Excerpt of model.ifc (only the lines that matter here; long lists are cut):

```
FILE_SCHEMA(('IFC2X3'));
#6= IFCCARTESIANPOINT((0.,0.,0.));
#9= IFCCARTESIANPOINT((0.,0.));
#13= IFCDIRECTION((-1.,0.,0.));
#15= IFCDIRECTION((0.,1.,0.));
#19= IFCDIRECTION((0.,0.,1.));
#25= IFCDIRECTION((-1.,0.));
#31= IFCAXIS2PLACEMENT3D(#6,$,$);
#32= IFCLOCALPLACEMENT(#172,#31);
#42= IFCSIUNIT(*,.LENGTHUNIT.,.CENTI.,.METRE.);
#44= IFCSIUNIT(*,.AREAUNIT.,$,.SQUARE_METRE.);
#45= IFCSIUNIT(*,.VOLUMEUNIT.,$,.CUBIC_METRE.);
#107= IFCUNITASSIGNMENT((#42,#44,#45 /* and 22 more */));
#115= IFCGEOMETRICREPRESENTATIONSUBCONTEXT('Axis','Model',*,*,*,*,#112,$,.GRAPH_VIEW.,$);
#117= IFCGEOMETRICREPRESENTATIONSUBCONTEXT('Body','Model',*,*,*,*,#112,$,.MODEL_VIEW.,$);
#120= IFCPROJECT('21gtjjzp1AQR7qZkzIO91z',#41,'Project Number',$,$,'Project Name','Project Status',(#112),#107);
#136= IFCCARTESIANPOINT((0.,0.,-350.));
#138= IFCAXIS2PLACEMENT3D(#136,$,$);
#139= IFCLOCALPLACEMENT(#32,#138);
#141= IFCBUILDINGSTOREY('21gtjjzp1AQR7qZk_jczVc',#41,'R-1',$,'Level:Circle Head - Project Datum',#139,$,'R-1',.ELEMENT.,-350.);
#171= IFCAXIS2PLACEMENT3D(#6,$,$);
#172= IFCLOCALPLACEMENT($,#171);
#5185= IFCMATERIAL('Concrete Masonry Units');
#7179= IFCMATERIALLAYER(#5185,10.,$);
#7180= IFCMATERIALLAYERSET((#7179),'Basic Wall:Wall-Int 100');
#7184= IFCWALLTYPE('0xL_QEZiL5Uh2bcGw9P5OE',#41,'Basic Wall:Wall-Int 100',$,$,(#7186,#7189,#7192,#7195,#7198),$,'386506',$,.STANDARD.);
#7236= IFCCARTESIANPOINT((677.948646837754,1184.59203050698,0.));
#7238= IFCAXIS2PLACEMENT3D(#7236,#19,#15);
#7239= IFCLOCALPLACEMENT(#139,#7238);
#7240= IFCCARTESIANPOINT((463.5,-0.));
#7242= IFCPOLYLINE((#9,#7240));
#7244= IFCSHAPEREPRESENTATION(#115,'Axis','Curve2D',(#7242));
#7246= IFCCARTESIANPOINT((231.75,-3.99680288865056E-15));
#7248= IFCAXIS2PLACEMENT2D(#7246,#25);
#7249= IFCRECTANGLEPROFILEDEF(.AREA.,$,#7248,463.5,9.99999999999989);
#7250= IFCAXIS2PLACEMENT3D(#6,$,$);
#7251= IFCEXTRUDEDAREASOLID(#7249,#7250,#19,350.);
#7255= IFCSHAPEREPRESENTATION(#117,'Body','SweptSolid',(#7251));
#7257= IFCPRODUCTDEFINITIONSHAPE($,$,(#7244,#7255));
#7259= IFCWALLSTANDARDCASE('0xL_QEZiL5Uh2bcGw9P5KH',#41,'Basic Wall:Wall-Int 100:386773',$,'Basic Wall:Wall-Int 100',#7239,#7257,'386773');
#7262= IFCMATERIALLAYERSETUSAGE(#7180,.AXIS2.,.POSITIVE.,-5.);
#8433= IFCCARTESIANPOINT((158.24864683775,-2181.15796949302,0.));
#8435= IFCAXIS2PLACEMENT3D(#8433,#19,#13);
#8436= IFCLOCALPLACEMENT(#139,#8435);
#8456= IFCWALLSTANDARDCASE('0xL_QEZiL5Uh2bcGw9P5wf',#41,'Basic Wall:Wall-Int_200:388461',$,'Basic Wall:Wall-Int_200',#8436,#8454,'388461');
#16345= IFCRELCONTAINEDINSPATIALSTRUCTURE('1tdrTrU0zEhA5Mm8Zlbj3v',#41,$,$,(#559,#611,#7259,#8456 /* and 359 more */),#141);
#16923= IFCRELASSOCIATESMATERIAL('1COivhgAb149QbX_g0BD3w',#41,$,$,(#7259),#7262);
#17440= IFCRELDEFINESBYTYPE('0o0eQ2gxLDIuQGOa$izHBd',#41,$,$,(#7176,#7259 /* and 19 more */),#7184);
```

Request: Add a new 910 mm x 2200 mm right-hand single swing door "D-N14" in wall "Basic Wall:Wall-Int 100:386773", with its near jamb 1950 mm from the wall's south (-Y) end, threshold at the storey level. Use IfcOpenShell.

```python
import numpy as np
import ifcopenshell
import ifcopenshell.api.feature
import ifcopenshell.api.geometry
import ifcopenshell.api.root
import ifcopenshell.api.spatial
import ifcopenshell.api.type
import ifcopenshell.geom
import ifcopenshell.util.element
import ifcopenshell.util.placement
import ifcopenshell.util.representation
import ifcopenshell.util.shape
import ifcopenshell.util.unit

model = ifcopenshell.open("model.ifc")
unit_scale = ifcopenshell.util.unit.calculate_unit_scale(model)
settings = ifcopenshell.geom.settings()


def volume(element):
    """Net volume in cubic metres, openings subtracted."""
    shape = ifcopenshell.geom.create_shape(settings, element)
    return ifcopenshell.util.shape.get_volume(shape.geometry)


wall = model.by_id(7259)
storey = ifcopenshell.util.element.get_container(wall, ifc_class="IfcBuildingStorey")
context = ifcopenshell.util.representation.get_context(model, "Model", "Body", "MODEL_VIEW")
before = volume(wall)

width, height, from_end, sill = 0.91, 2.2, 1.95, 0.0  # metres

# The wall runs along its own X axis, and the end named is its -X end.
wall_shape = ifcopenshell.geom.create_shape(settings, wall)
x, y, z = ifcopenshell.util.shape.get_vertices(wall_shape.geometry).T
start = x.min() + from_end
face, thickness = float(y.min()), float(y.max() - y.min())
wall_matrix = ifcopenshell.util.placement.get_local_placement(wall.ObjectPlacement)
level = ifcopenshell.util.placement.get_local_placement(storey.ObjectPlacement)[2, 3]


def in_wall(x, y):
    """Placement at x, y metres in the wall's axes, at sill height."""
    matrix = wall_matrix.copy()
    matrix[:, 3] = wall_matrix @ np.array([x / unit_scale, y / unit_scale, 0.0, 1.0])
    matrix[2, 3] = level + sill / unit_scale
    return matrix


# Opening: a box that overshoots both wall faces by 50 mm.
opening = ifcopenshell.api.root.create_entity(model, ifc_class="IfcOpeningElement")
box = ifcopenshell.api.geometry.add_wall_representation(
    model, context=context, length=width, height=height, thickness=thickness + 0.1
)
ifcopenshell.api.geometry.assign_representation(model, product=opening, representation=box)
ifcopenshell.api.geometry.edit_object_placement(model, product=opening, matrix=in_wall(start, face - 0.05), is_si=False)
ifcopenshell.api.feature.add_feature(model, feature=opening, element=wall)

door = ifcopenshell.api.root.create_entity(model, ifc_class="IfcDoor", name="D-N14")
door.OverallWidth, door.OverallHeight = width / unit_scale, height / unit_scale
body = ifcopenshell.api.geometry.add_door_representation(
    model,
    context=context,
    overall_width=door.OverallWidth,
    overall_height=door.OverallHeight,
    operation_type="SINGLE_SWING_RIGHT",
    lining_properties={"LiningDepth": thickness / unit_scale, "ThresholdDepth": thickness / unit_scale},
)
ifcopenshell.api.geometry.assign_representation(model, product=door, representation=body)
ifcopenshell.api.spatial.assign_container(model, products=[door], relating_structure=storey)
fills = ifcopenshell.api.feature.add_filling(model, opening=opening, element=door)
fills.OwnerHistory = door.OwnerHistory  # required in IFC2X3

# IFC2X3 keeps the operation on the door style.
style = ifcopenshell.api.root.create_entity(model, ifc_class="IfcDoorStyle", name="D-N14")
style.OperationType, style.ConstructionType = "SINGLE_SWING_RIGHT", "NOTDEFINED"
style.ParameterTakesPrecedence = style.Sizeable = False
ifcopenshell.api.type.assign_type(model, related_objects=[door], relating_type=style)

# The lining spans the wall, so the door starts at the wall face.
ifcopenshell.api.geometry.edit_object_placement(model, product=door, matrix=in_wall(start, face), is_si=False)

after = volume(wall)

print(f"wall volume {before:.3f} -> {after:.3f} m3")

model.write("model_updated.ifc")
```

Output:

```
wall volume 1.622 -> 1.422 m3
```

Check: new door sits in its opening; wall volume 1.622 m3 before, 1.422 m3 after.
